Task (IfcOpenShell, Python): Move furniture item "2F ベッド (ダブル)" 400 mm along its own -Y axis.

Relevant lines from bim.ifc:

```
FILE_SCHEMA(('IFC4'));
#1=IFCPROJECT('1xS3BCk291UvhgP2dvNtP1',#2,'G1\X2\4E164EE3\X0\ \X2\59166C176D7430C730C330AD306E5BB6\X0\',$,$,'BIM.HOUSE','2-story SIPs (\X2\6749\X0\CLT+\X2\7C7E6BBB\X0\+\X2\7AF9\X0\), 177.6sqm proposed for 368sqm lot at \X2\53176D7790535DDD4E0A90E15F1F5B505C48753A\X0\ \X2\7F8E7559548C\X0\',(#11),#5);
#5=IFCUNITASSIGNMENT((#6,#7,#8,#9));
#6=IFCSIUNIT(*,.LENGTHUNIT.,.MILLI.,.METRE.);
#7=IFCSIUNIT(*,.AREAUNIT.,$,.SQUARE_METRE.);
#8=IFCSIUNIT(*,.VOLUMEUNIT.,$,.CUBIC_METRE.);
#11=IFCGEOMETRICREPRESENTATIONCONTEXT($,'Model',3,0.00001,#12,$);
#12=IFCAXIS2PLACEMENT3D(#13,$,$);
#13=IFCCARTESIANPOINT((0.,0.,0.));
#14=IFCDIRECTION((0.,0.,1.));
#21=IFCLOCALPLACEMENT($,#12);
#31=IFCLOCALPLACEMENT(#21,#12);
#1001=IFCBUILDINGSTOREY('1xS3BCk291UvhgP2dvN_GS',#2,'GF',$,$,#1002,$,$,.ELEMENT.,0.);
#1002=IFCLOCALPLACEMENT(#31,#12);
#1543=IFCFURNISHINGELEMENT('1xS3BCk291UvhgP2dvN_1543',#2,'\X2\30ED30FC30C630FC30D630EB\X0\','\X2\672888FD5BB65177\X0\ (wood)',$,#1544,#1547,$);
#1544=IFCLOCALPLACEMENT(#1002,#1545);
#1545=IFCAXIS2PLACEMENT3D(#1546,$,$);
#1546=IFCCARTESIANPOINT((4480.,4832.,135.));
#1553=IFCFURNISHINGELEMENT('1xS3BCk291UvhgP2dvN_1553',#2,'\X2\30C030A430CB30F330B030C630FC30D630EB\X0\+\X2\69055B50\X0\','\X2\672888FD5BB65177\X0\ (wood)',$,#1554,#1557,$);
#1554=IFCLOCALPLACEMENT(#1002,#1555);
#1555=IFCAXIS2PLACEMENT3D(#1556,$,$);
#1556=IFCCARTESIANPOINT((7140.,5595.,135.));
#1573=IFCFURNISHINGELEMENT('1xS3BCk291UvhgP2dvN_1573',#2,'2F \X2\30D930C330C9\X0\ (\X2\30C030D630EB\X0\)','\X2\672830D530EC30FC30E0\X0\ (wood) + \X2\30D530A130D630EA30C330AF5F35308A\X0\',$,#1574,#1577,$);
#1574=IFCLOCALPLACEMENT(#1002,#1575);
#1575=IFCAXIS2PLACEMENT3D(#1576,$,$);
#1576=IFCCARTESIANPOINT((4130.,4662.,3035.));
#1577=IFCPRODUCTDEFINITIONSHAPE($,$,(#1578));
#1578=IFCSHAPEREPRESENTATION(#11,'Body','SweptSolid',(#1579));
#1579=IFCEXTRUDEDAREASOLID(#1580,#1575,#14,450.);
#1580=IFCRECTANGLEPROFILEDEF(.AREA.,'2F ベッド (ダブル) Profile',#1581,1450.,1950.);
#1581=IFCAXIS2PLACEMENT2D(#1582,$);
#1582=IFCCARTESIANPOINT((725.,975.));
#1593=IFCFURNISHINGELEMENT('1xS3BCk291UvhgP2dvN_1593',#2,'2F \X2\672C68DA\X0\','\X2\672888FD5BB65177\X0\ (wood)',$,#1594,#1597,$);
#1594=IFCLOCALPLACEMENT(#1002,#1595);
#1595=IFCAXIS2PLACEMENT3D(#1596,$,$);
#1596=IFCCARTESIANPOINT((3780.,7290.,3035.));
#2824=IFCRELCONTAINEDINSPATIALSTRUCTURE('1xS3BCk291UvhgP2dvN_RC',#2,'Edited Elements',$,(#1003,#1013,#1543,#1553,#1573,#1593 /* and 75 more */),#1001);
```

```python
import ifcopenshell
import ifcopenshell.api.geometry
import ifcopenshell.util.placement
import ifcopenshell.util.unit

model = ifcopenshell.open("bim.ifc")
unit_scale = ifcopenshell.util.unit.calculate_unit_scale(model)

item = model.by_guid("1xS3BCk291UvhgP2dvN_1573")
matrix = ifcopenshell.util.placement.get_local_placement(item.ObjectPlacement)
matrix[:3, 3] -= matrix[:3, 1] * 0.4 / unit_scale
ifcopenshell.api.geometry.edit_object_placement(model, product=item, matrix=matrix, is_si=False)

print(ifcopenshell.util.placement.get_local_placement(item.ObjectPlacement).round(3) + 0.0)

model.write("bim_v2.ifc")
```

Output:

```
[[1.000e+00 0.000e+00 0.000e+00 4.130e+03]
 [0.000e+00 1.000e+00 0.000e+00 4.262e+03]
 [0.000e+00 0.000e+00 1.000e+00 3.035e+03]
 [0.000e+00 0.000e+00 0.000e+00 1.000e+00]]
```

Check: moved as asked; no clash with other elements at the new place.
